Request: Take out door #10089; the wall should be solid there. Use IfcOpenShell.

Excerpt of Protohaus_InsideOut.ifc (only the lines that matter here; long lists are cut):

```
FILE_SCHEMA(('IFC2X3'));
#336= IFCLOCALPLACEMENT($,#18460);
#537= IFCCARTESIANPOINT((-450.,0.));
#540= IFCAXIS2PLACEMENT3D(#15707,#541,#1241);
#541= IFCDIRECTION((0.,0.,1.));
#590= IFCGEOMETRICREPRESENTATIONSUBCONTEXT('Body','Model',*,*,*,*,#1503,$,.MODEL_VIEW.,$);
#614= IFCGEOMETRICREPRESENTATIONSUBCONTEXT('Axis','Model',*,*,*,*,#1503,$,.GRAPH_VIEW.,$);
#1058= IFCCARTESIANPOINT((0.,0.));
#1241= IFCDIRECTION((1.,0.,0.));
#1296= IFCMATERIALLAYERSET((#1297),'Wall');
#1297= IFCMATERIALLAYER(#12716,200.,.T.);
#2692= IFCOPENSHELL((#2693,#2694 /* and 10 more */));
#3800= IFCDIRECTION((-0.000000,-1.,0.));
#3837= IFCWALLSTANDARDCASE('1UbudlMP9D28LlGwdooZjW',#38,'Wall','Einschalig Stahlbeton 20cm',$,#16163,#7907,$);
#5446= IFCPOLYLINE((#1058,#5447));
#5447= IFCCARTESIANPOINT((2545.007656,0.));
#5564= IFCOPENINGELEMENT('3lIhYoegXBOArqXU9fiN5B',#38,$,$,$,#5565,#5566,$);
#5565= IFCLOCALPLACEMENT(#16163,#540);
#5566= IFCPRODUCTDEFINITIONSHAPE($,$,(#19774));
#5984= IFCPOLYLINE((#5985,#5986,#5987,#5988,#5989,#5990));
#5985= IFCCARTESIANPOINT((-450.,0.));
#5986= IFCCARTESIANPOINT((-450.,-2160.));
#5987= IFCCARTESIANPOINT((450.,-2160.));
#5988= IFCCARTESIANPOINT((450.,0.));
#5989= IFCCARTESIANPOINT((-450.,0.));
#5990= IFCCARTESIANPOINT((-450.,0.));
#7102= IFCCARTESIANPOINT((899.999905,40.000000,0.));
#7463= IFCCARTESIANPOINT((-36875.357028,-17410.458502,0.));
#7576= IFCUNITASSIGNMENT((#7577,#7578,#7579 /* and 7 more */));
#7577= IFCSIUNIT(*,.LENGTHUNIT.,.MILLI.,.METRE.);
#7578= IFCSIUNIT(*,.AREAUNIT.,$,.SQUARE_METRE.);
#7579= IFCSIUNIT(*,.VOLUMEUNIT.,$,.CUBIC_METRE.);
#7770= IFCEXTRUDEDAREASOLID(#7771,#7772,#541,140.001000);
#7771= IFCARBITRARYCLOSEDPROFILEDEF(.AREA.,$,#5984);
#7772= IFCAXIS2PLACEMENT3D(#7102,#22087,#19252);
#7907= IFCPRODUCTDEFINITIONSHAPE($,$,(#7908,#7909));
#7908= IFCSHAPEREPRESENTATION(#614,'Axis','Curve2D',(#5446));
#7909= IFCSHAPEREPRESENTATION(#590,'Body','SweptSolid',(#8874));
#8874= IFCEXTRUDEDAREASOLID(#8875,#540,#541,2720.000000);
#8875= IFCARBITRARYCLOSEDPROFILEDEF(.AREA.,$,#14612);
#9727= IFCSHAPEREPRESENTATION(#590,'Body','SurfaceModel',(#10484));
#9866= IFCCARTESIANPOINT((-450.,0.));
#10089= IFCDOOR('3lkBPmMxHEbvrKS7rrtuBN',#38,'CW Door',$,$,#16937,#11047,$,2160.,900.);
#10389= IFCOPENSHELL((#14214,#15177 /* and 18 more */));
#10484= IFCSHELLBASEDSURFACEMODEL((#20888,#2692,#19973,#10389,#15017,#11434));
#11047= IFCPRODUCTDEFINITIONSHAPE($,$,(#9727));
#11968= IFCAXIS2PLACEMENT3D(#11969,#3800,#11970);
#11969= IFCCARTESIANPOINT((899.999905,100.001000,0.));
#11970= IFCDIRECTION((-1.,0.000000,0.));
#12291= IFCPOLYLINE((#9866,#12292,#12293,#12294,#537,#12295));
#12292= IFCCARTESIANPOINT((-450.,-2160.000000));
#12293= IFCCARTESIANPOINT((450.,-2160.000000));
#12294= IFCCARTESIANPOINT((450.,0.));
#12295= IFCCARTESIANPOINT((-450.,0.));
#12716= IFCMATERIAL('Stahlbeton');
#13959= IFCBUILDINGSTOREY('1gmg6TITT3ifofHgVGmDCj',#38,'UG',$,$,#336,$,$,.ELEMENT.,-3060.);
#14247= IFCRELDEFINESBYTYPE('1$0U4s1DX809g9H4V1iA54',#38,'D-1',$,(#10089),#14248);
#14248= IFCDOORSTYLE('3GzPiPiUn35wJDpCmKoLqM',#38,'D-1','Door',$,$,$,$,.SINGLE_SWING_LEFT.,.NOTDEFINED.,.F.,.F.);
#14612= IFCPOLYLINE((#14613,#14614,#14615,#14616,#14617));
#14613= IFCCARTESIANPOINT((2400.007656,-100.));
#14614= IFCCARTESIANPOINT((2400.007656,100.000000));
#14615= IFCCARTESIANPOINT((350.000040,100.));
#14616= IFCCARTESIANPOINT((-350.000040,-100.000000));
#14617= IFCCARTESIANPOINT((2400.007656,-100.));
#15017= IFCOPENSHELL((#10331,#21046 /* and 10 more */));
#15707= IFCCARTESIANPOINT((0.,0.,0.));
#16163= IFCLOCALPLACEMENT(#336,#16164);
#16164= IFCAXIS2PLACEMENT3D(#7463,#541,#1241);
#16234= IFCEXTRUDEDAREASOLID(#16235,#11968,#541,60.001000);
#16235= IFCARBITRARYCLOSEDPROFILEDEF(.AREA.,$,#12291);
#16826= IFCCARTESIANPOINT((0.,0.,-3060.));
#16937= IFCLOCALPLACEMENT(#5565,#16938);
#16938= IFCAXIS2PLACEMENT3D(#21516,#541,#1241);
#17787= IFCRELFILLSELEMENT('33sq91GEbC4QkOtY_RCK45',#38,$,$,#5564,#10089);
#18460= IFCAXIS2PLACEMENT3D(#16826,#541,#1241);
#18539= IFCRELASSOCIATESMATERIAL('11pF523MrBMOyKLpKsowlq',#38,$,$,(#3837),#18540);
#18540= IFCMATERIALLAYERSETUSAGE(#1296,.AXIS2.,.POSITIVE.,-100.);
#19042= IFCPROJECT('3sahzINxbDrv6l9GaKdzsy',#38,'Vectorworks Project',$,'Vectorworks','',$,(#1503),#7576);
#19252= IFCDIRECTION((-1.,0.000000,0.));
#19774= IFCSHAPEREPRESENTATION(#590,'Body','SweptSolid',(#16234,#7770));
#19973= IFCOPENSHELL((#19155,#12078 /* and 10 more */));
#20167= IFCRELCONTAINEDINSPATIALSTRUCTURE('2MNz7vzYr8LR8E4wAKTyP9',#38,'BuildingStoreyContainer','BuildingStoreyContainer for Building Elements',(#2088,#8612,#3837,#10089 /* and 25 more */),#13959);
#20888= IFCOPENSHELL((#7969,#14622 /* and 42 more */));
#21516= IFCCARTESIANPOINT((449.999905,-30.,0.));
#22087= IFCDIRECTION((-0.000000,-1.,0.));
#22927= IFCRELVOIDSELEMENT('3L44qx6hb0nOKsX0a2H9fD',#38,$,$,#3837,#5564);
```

```python
import ifcopenshell
import ifcopenshell.api.feature
import ifcopenshell.api.root
import ifcopenshell.geom
import ifcopenshell.util.shape

model = ifcopenshell.open("Protohaus_InsideOut.ifc")
settings = ifcopenshell.geom.settings()


def volume(element):
    """Net volume in cubic metres, openings subtracted."""
    shape = ifcopenshell.geom.create_shape(settings, element)
    return ifcopenshell.util.shape.get_volume(shape.geometry)


door = model.by_id(10089)
opening = door.FillsVoids[0].RelatingOpeningElement
wall = opening.VoidsElements[0].RelatingBuildingElement
before = volume(wall)

ifcopenshell.api.root.remove_product(model, product=door)
ifcopenshell.api.feature.remove_feature(model, feature=opening)

after = volume(wall)

print(f"wall volume {before:.3f} -> {after:.3f} m3")

model.write("Protohaus_InsideOut_edited.ifc")
```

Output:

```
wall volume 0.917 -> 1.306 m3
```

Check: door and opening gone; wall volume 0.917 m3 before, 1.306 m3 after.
